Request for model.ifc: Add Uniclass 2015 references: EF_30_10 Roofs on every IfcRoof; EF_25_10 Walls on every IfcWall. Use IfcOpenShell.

First a look at what the model holds.

```python
import ifcopenshell

model = ifcopenshell.open("model.ifc")
print(model.schema)
print("classifications:", [c.Name for c in model.by_type("IfcClassification")])
for ifc_class in ("IfcDoor", "IfcRoof", "IfcStair", "IfcWall", "IfcWindow"):
    print(ifc_class, len(model.by_type(ifc_class)))
```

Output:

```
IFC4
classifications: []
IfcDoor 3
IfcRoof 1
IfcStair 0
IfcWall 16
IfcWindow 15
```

```python
import ifcopenshell
import ifcopenshell.api.classification

model = ifcopenshell.open("model.ifc")

system = ifcopenshell.api.classification.add_classification(model, classification="Uniclass 2015")

codes = {
    "IfcRoof": ("EF_30_10", "Roofs"),
    "IfcWall": ("EF_25_10", "Walls"),
}
for ifc_class, (code, name) in codes.items():
    products = model.by_type(ifc_class)
    ifcopenshell.api.classification.add_reference(
        model, products=products, classification=system, identification=code, name=name
    )
    print(code, len(products))

model.write("model-out.ifc")
```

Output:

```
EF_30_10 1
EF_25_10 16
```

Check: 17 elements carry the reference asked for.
